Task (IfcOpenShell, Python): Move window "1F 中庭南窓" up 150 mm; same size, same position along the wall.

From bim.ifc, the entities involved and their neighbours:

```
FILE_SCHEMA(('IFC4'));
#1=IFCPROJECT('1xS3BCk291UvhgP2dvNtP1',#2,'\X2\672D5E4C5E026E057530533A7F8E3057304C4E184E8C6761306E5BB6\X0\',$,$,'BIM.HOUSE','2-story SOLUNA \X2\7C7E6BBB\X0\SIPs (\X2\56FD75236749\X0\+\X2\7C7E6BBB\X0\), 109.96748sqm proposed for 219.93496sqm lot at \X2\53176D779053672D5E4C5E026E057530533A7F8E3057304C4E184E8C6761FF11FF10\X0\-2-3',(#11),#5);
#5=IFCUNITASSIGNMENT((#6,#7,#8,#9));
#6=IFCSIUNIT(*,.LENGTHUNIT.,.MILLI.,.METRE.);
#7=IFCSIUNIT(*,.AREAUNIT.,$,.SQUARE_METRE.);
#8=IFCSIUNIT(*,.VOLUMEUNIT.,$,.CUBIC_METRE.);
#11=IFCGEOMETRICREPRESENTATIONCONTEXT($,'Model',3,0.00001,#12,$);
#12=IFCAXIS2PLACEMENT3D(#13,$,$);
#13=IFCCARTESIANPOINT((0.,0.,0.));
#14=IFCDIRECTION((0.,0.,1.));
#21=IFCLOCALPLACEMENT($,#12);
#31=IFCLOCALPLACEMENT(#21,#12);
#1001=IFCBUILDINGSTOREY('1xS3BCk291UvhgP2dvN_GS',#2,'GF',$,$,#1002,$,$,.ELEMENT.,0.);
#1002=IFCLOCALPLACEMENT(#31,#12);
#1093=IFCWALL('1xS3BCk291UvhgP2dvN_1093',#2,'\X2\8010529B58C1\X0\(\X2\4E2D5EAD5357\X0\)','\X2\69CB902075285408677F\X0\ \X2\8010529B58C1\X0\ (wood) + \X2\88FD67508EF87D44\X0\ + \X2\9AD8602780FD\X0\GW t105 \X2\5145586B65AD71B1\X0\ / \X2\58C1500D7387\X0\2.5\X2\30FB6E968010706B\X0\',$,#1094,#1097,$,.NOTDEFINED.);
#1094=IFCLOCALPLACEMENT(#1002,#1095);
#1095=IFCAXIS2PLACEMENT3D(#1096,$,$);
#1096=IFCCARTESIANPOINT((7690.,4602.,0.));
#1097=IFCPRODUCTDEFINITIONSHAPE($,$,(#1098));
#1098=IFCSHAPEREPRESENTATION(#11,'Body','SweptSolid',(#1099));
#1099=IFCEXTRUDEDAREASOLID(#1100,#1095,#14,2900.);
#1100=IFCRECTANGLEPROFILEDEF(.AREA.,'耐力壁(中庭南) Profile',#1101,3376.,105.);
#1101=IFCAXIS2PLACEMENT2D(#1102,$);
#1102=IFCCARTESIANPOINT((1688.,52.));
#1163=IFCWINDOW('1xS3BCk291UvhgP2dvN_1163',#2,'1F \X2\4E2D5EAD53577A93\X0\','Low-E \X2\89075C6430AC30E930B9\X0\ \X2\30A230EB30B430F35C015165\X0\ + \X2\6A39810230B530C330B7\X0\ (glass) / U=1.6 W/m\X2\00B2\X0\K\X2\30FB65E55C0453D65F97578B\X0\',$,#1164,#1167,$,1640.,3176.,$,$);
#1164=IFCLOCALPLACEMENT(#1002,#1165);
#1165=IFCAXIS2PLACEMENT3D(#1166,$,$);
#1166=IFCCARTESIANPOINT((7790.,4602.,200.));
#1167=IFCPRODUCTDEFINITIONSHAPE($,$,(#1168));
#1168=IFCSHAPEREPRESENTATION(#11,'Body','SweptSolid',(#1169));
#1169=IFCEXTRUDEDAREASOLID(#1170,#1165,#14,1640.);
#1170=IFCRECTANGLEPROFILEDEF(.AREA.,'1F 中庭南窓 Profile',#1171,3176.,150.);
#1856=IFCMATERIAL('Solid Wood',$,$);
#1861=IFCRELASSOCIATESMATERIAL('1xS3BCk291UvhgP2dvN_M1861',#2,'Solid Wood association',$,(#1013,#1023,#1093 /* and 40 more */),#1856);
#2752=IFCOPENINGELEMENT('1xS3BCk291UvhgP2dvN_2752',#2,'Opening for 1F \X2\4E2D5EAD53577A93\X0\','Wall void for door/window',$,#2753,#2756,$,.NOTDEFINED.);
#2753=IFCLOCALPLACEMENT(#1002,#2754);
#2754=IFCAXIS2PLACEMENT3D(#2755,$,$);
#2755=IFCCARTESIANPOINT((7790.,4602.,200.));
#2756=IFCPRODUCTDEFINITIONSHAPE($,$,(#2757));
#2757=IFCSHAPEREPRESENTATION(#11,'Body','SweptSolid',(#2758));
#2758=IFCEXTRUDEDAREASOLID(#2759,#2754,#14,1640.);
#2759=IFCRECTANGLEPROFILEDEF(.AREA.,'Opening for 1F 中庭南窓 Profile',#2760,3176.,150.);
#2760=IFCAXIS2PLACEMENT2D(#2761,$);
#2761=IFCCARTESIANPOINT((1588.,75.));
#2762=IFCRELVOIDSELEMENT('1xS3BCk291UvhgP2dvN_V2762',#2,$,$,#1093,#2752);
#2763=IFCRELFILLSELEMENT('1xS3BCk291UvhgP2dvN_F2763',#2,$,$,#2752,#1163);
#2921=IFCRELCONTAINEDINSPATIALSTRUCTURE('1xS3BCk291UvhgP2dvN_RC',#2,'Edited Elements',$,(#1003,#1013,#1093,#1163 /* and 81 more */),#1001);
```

```python
import numpy as np
import ifcopenshell
import ifcopenshell.api.geometry
import ifcopenshell.util.placement
import ifcopenshell.util.unit

model = ifcopenshell.open("bim.ifc")
unit_scale = ifcopenshell.util.unit.calculate_unit_scale(model)

window = model.by_id(1163)
opening = window.FillsVoids[0].RelatingOpeningElement
dz = 0.15 / unit_scale

shift = np.array([0.0, 0.0, dz])
# The window is not placed relative to its opening, so move both.
for product in (opening, window):
    matrix = ifcopenshell.util.placement.get_local_placement(product.ObjectPlacement)
    matrix[:3, 3] += shift
    ifcopenshell.api.geometry.edit_object_placement(model, product=product, matrix=matrix, is_si=False)

print(f"moved by {dz * unit_scale:+.3f} m")

model.write("bim_v2.ifc")
```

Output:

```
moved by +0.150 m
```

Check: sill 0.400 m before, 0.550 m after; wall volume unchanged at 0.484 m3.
